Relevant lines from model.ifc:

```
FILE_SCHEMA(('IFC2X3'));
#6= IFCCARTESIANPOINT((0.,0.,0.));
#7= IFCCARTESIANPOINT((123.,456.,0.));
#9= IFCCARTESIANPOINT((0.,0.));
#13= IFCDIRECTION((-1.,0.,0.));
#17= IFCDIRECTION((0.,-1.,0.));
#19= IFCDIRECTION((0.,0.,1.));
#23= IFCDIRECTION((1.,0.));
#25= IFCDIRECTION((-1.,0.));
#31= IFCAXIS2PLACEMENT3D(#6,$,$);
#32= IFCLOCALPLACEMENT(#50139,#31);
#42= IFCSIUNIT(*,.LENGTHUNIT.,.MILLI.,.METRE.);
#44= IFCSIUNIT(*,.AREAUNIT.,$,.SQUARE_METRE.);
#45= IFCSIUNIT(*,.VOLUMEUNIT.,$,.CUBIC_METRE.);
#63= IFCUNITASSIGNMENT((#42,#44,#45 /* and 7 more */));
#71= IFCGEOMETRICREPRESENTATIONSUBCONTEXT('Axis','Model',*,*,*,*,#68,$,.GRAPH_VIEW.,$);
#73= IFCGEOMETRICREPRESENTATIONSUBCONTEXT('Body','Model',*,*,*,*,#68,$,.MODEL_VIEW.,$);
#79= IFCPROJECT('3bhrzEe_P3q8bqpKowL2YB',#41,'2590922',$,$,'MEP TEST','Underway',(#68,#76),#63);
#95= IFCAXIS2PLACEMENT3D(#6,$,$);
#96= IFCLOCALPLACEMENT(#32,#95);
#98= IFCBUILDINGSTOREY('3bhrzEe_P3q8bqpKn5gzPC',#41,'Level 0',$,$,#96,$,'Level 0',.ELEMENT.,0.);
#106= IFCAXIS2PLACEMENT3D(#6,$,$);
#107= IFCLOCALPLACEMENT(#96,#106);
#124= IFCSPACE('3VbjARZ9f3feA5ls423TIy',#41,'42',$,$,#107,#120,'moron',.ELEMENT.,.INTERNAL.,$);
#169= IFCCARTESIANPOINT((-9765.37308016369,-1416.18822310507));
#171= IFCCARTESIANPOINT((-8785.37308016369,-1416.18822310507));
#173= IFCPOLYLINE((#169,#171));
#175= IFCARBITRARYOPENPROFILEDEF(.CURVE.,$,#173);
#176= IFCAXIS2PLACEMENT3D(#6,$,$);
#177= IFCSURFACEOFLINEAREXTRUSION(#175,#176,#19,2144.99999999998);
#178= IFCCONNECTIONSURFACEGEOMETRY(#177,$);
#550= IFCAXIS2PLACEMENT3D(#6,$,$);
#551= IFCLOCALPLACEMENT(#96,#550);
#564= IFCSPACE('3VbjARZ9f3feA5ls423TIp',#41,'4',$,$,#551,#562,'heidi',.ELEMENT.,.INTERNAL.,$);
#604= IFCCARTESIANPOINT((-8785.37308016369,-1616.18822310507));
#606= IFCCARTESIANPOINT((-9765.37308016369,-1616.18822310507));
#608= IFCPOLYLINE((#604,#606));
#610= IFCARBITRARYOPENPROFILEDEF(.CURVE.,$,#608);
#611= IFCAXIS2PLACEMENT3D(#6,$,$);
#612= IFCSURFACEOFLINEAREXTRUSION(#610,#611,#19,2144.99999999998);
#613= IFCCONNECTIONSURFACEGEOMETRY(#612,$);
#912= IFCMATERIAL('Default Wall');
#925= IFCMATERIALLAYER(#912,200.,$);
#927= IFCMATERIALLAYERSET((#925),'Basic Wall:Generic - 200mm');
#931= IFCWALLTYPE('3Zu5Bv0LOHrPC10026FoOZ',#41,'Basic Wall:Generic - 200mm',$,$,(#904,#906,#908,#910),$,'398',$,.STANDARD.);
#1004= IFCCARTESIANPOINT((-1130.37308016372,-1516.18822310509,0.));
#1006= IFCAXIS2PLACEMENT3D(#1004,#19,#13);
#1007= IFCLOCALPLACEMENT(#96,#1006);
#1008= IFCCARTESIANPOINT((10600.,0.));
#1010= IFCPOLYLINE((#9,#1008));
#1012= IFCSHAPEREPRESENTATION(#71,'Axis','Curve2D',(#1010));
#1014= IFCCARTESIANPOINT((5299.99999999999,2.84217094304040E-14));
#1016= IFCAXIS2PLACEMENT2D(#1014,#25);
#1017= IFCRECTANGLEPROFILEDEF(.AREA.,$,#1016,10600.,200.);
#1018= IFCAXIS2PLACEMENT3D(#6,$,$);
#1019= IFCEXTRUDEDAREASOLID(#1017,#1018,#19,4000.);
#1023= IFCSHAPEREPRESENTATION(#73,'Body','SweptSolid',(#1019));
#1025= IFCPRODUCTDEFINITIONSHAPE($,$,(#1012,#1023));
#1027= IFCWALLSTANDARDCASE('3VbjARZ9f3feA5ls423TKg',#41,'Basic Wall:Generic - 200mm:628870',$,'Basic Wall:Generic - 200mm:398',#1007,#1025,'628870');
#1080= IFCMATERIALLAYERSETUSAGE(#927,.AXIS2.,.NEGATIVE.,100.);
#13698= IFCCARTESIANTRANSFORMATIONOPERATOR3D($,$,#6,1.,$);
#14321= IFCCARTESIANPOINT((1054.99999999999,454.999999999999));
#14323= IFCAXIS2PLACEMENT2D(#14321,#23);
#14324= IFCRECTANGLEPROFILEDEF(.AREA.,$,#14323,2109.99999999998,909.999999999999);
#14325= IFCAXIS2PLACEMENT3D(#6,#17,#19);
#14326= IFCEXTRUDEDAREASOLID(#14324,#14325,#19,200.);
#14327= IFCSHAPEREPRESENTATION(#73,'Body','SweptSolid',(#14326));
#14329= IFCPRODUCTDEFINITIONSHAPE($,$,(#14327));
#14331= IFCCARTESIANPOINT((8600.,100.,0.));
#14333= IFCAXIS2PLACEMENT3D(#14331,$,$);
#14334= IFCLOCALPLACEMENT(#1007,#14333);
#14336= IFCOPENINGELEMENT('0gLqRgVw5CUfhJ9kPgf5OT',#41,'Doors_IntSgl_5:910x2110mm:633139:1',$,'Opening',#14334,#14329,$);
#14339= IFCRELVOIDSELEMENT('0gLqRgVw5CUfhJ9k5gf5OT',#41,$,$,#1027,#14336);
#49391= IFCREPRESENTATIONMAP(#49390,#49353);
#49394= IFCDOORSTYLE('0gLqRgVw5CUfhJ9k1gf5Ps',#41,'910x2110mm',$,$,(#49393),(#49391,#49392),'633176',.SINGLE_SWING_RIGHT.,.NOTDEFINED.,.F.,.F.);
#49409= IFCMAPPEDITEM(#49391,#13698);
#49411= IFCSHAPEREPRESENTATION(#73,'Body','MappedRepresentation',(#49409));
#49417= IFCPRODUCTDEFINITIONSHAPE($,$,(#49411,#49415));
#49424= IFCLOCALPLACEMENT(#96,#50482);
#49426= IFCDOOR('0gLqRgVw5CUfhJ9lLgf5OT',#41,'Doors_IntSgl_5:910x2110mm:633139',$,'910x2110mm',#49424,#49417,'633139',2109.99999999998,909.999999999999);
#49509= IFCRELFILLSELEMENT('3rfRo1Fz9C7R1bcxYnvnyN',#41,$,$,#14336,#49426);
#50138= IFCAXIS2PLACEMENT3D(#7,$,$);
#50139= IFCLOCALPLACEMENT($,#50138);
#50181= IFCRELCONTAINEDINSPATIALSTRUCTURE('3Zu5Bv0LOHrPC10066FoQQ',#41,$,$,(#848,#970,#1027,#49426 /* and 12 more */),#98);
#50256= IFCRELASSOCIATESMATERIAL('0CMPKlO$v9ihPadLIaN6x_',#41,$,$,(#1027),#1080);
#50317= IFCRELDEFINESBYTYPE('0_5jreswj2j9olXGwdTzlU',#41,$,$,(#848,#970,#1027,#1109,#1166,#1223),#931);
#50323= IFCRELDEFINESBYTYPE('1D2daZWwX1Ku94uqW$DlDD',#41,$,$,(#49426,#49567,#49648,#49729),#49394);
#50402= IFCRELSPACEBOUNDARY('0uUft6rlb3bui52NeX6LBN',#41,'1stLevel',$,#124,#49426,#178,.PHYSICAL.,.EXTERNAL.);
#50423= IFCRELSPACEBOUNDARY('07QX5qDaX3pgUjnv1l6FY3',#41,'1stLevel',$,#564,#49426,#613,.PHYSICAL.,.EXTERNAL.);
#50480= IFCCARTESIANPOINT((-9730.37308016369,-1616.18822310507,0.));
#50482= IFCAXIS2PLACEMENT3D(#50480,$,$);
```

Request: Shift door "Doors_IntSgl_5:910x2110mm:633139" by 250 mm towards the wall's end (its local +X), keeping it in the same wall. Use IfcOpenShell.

```python
import numpy as np
import ifcopenshell
import ifcopenshell.api.geometry
import ifcopenshell.util.placement
import ifcopenshell.util.unit

model = ifcopenshell.open("model.ifc")
unit_scale = ifcopenshell.util.unit.calculate_unit_scale(model)

door = model.by_id(49426)
opening = door.FillsVoids[0].RelatingOpeningElement
wall = opening.VoidsElements[0].RelatingBuildingElement

wall_matrix = ifcopenshell.util.placement.get_local_placement(wall.ObjectPlacement)
shift = wall_matrix[:3, 0] * 0.25 / unit_scale
before = ifcopenshell.util.placement.get_local_placement(door.ObjectPlacement)[:3, 3].copy()

# The door is not placed relative to its opening, so move both.
for product in (opening, door):
    matrix = ifcopenshell.util.placement.get_local_placement(product.ObjectPlacement)
    matrix[:3, 3] += shift
    ifcopenshell.api.geometry.edit_object_placement(model, product=product, matrix=matrix, is_si=False)

# Space boundary surfaces are stored in each space's coordinates; move them too.
for rel in door.ProvidesBoundaries:
    if not rel.ConnectionGeometry:
        continue
    surface = rel.ConnectionGeometry.SurfaceOnRelatingElement
    space_matrix = ifcopenshell.util.placement.get_local_placement(rel.RelatingSpace.ObjectPlacement)
    point = np.array(surface.Position.Location.Coordinates) + space_matrix[:3, :3].T @ shift
    surface.Position = model.createIfcAxis2Placement3D(
        model.createIfcCartesianPoint(point.tolist()), surface.Position.Axis, surface.Position.RefDirection
    )

after = ifcopenshell.util.placement.get_local_placement(door.ObjectPlacement)[:3, 3]
print("door moved by", (after - before).round(3) + 0.0)

model.write("model-out.ifc")
```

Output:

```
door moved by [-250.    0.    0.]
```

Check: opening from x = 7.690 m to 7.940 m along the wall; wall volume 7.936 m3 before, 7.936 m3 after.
